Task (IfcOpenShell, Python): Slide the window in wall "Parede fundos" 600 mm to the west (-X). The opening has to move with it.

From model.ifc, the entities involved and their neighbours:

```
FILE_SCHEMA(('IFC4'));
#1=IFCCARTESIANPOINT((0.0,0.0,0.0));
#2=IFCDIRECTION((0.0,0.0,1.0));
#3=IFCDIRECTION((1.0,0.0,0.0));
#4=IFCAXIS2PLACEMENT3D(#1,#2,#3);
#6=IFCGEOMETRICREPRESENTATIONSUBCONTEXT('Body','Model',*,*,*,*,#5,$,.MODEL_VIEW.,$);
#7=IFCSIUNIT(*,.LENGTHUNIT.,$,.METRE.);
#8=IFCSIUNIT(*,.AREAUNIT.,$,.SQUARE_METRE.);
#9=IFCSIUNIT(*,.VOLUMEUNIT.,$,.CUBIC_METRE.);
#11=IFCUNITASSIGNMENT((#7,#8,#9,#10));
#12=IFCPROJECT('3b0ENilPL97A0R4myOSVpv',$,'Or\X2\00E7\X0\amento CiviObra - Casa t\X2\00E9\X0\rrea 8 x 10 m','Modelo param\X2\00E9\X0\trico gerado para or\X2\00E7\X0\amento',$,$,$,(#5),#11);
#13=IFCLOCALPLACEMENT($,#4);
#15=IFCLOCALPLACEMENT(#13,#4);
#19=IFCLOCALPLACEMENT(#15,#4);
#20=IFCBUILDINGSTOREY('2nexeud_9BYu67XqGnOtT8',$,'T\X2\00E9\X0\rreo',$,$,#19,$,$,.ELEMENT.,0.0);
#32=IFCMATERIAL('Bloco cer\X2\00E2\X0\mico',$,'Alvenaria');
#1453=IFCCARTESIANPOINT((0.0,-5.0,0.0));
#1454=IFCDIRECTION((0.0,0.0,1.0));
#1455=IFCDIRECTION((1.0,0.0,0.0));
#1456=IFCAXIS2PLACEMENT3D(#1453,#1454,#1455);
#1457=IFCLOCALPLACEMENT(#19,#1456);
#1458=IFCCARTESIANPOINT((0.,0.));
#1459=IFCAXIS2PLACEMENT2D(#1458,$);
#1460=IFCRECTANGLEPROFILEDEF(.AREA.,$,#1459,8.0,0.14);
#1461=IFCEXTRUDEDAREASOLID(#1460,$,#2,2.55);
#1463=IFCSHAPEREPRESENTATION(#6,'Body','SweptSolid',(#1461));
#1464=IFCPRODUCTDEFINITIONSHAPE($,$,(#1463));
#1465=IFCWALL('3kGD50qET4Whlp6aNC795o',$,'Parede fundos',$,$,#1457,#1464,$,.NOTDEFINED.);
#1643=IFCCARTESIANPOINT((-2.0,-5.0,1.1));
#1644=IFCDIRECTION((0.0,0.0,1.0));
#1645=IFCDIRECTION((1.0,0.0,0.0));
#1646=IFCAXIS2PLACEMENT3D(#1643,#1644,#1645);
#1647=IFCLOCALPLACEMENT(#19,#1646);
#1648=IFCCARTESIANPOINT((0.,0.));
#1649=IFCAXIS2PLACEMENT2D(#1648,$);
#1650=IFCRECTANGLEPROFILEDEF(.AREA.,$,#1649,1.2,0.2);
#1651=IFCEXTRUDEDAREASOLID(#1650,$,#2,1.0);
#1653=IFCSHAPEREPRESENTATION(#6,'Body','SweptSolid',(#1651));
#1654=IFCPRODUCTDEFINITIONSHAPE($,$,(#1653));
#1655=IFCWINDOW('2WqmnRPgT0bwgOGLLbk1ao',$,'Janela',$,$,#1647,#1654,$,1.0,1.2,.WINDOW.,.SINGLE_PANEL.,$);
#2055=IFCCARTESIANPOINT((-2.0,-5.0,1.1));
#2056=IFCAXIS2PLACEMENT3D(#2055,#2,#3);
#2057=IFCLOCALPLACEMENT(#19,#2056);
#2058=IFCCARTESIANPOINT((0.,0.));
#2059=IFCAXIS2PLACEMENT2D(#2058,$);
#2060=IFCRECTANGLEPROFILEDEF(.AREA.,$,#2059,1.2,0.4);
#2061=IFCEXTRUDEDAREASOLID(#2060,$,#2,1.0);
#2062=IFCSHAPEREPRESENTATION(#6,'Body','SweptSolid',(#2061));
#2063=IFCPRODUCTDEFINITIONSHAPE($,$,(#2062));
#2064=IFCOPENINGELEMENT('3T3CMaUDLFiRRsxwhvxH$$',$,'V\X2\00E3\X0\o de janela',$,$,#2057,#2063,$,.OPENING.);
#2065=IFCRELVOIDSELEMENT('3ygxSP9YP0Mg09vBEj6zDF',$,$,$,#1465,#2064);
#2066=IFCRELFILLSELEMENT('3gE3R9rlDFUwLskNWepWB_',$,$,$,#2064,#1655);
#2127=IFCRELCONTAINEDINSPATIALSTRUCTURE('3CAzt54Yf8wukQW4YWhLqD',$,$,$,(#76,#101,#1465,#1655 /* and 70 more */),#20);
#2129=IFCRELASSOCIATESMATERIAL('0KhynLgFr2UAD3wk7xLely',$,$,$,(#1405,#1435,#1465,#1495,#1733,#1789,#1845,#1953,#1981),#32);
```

```python
import ifcopenshell
import ifcopenshell.api.geometry
import ifcopenshell.util.placement
import ifcopenshell.util.unit

model = ifcopenshell.open("model.ifc")
unit_scale = ifcopenshell.util.unit.calculate_unit_scale(model)

window = model.by_id(1655)
opening = window.FillsVoids[0].RelatingOpeningElement
wall = opening.VoidsElements[0].RelatingBuildingElement

wall_matrix = ifcopenshell.util.placement.get_local_placement(wall.ObjectPlacement)
shift = wall_matrix[:3, 0] * -0.6 / unit_scale
before = ifcopenshell.util.placement.get_local_placement(window.ObjectPlacement)[:3, 3].copy()

# The window is not placed relative to its opening, so move both.
for product in (opening, window):
    matrix = ifcopenshell.util.placement.get_local_placement(product.ObjectPlacement)
    matrix[:3, 3] += shift
    ifcopenshell.api.geometry.edit_object_placement(model, product=product, matrix=matrix, is_si=False)

after = ifcopenshell.util.placement.get_local_placement(window.ObjectPlacement)[:3, 3]
print("window moved by", (after - before).round(3) + 0.0)

model.write("model_edited.ifc")
```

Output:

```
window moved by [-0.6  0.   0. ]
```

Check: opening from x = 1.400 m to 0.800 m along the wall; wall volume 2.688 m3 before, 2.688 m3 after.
